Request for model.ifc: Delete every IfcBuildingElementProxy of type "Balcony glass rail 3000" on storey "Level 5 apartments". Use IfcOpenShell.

First a look at what the model holds.

```python
import ifcopenshell
import ifcopenshell.util.element

model = ifcopenshell.open("model.ifc")
print(model.schema)
storey = next(s for s in model.by_type("IfcBuildingStorey") if s.Name == "Level 5 apartments")
proxies = [e for e in ifcopenshell.util.element.get_decomposition(storey) if e.is_a("IfcBuildingElementProxy")]
seen = {}
for e in proxies:
    element_type = ifcopenshell.util.element.get_type(e)
    name = element_type.Name if element_type not in (None, e) else None
    seen[name] = seen.get(name, 0) + 1
for name, count in sorted(seen.items(), key=str):
    print(count, "x", name)
```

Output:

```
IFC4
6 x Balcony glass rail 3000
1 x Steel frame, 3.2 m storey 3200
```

```python
import ifcopenshell
import ifcopenshell.api.root
import ifcopenshell.util.element

model = ifcopenshell.open("model.ifc")

storey = next(s for s in model.by_type("IfcBuildingStorey") if s.Name == "Level 5 apartments")
proxies = [e for e in ifcopenshell.util.element.get_decomposition(storey) if e.is_a("IfcBuildingElementProxy")]
targets = [e for e in proxies if (t := ifcopenshell.util.element.get_type(e)) not in (None, e) and t.Name == "Balcony glass rail 3000"]

for e in targets:
    ifcopenshell.api.root.remove_product(model, product=e)
print(len(targets), "removed")

model.write("model_rev.ifc")
```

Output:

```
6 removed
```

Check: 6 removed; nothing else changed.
